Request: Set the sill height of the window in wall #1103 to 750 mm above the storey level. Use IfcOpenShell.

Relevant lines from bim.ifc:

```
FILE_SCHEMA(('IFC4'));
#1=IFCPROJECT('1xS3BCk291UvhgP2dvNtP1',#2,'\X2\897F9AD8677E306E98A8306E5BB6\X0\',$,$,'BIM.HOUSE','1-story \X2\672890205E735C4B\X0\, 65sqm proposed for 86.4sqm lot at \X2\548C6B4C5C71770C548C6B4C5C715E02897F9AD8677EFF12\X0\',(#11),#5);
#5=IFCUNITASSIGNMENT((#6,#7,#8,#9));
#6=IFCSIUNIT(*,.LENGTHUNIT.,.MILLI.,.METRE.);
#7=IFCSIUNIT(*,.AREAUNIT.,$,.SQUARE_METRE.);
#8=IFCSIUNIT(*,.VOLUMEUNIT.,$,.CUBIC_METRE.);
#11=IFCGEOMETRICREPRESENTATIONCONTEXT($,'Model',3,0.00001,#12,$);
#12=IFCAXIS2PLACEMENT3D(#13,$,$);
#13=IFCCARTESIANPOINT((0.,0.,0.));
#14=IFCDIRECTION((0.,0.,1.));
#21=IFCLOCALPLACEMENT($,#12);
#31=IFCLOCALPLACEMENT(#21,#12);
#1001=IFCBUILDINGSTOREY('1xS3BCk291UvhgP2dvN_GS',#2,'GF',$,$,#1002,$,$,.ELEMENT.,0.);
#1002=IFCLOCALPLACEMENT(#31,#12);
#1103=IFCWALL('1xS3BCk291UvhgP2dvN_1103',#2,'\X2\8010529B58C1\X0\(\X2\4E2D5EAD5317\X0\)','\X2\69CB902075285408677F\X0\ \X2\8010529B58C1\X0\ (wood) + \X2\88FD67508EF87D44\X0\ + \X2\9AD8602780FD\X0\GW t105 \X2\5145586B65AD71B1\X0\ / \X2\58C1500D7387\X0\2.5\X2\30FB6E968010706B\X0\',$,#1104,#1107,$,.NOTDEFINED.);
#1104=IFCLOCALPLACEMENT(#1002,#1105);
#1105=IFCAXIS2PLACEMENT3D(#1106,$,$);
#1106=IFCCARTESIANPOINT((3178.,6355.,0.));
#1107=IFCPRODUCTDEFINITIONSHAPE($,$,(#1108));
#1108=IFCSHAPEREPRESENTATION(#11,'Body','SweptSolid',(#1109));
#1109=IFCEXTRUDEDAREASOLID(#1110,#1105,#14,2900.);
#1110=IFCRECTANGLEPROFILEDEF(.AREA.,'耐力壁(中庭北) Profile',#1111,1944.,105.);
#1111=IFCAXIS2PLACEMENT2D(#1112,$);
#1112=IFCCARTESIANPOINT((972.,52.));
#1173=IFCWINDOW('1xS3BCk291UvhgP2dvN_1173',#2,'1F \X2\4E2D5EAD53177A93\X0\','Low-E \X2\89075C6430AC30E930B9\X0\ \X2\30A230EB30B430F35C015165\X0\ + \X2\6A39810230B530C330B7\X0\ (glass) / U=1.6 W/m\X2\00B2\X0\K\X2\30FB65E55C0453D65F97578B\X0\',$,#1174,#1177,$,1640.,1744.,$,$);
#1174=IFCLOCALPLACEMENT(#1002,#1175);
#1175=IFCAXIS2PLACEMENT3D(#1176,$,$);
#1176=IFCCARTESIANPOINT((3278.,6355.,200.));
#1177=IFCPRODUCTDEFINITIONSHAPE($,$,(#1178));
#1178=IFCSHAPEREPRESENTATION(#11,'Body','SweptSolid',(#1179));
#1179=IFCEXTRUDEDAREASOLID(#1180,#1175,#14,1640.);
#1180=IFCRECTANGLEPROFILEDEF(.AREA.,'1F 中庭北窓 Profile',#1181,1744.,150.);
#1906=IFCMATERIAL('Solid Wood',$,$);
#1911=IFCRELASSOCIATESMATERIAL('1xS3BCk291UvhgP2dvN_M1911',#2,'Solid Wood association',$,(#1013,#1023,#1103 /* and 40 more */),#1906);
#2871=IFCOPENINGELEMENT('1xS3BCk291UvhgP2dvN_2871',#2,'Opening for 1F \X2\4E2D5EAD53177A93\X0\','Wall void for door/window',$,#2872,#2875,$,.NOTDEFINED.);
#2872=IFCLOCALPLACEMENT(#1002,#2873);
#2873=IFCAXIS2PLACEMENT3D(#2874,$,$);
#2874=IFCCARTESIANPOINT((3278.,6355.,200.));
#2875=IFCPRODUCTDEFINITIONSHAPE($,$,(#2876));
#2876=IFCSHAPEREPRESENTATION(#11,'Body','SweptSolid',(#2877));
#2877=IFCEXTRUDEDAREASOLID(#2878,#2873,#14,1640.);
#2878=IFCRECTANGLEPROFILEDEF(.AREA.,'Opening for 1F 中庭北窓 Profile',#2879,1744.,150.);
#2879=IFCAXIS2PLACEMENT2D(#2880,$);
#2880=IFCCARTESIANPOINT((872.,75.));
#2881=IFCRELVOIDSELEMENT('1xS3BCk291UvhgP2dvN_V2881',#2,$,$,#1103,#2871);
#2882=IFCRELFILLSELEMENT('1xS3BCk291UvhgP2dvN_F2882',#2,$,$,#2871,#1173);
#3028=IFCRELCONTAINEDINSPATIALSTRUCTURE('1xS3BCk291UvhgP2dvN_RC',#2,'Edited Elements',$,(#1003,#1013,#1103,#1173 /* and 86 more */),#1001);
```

```python
import numpy as np
import ifcopenshell
import ifcopenshell.api.geometry
import ifcopenshell.geom
import ifcopenshell.util.element
import ifcopenshell.util.placement
import ifcopenshell.util.shape
import ifcopenshell.util.unit

model = ifcopenshell.open("bim.ifc")
unit_scale = ifcopenshell.util.unit.calculate_unit_scale(model)

window = model.by_guid("1xS3BCk291UvhgP2dvN_1173")
opening = window.FillsVoids[0].RelatingOpeningElement
storey = ifcopenshell.util.element.get_container(window, ifc_class="IfcBuildingStorey")
level = ifcopenshell.util.placement.get_local_placement(storey.ObjectPlacement)[2, 3]

# The opening's origin need not be at the sill, so measure its lowest point.
shape = ifcopenshell.geom.create_shape(ifcopenshell.geom.settings(), opening)
bottom = ifcopenshell.util.shape.get_shape_bottom_elevation(shape, shape.geometry) / unit_scale
dz = level + 750.0 - bottom

shift = np.array([0.0, 0.0, dz])
# The window is not placed relative to its opening, so move both.
for product in (opening, window):
    matrix = ifcopenshell.util.placement.get_local_placement(product.ObjectPlacement)
    matrix[:3, 3] += shift
    ifcopenshell.api.geometry.edit_object_placement(model, product=product, matrix=matrix, is_si=False)

print(f"moved by {dz * unit_scale:+.3f} m")

model.write("bim-out.ifc")
```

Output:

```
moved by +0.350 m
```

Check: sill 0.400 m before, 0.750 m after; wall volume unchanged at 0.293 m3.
